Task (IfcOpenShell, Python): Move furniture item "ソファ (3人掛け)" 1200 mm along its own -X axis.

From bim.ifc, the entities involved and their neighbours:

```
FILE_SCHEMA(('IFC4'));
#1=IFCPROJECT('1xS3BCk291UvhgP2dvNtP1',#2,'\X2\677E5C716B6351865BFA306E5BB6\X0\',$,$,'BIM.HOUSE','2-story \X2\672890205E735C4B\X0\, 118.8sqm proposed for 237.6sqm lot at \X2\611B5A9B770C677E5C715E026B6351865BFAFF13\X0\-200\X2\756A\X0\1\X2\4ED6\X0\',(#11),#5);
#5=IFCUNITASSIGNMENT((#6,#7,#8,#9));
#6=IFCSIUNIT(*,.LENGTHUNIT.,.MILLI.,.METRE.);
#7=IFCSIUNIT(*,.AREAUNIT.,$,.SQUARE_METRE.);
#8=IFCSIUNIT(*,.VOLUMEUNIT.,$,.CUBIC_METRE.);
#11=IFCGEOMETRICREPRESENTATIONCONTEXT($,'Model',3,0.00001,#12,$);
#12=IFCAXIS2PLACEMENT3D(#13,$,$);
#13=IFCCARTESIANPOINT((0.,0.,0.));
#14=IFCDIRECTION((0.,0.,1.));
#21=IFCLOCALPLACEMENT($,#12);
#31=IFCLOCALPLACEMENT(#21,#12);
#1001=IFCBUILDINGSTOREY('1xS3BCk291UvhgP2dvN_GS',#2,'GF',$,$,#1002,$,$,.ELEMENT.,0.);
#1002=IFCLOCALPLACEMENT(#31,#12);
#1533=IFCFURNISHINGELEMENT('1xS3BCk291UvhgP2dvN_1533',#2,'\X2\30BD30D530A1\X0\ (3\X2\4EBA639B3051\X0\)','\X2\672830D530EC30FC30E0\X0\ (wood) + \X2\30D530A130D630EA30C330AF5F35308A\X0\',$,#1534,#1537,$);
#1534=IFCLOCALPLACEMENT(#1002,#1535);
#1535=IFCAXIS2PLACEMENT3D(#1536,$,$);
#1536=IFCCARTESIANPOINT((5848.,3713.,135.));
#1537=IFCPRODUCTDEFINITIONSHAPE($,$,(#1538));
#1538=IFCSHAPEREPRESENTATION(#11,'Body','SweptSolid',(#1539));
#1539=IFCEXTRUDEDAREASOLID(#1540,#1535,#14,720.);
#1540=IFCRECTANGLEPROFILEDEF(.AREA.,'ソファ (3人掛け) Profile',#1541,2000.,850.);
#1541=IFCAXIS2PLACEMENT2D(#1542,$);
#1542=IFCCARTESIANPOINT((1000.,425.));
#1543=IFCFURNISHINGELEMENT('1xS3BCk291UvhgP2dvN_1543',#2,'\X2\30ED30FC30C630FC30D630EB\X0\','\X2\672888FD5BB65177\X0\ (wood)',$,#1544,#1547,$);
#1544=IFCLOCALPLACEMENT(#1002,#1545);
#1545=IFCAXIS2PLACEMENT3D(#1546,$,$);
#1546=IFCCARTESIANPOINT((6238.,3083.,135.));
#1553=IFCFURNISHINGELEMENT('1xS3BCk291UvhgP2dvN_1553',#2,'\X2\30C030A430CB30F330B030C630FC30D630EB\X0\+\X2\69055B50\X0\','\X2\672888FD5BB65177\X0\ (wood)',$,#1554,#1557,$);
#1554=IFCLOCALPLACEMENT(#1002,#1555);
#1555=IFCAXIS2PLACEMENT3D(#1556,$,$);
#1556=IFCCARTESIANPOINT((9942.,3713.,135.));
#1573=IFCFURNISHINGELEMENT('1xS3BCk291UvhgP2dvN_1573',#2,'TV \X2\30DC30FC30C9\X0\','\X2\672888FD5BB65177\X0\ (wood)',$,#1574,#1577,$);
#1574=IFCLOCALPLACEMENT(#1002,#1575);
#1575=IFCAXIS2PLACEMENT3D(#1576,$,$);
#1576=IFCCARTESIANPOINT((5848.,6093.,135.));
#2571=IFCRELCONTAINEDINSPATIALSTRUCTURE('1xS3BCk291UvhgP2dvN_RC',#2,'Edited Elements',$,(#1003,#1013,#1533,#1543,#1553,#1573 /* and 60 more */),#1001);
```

```python
import ifcopenshell
import ifcopenshell.api.geometry
import ifcopenshell.util.placement

model = ifcopenshell.open("bim.ifc")

item = model.by_guid("1xS3BCk291UvhgP2dvN_1533")
matrix = ifcopenshell.util.placement.get_local_placement(item.ObjectPlacement)
matrix[:3, 3] -= matrix[:3, 0] * 1200.0
ifcopenshell.api.geometry.edit_object_placement(model, product=item, matrix=matrix, is_si=False)

print(ifcopenshell.util.placement.get_local_placement(item.ObjectPlacement).round(3) + 0.0)

model.write("bim_rev.ifc")
```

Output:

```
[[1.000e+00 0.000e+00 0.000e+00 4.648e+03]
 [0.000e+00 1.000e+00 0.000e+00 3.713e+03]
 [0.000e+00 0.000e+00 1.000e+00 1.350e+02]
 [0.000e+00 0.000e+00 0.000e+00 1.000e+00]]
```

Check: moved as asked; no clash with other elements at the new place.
